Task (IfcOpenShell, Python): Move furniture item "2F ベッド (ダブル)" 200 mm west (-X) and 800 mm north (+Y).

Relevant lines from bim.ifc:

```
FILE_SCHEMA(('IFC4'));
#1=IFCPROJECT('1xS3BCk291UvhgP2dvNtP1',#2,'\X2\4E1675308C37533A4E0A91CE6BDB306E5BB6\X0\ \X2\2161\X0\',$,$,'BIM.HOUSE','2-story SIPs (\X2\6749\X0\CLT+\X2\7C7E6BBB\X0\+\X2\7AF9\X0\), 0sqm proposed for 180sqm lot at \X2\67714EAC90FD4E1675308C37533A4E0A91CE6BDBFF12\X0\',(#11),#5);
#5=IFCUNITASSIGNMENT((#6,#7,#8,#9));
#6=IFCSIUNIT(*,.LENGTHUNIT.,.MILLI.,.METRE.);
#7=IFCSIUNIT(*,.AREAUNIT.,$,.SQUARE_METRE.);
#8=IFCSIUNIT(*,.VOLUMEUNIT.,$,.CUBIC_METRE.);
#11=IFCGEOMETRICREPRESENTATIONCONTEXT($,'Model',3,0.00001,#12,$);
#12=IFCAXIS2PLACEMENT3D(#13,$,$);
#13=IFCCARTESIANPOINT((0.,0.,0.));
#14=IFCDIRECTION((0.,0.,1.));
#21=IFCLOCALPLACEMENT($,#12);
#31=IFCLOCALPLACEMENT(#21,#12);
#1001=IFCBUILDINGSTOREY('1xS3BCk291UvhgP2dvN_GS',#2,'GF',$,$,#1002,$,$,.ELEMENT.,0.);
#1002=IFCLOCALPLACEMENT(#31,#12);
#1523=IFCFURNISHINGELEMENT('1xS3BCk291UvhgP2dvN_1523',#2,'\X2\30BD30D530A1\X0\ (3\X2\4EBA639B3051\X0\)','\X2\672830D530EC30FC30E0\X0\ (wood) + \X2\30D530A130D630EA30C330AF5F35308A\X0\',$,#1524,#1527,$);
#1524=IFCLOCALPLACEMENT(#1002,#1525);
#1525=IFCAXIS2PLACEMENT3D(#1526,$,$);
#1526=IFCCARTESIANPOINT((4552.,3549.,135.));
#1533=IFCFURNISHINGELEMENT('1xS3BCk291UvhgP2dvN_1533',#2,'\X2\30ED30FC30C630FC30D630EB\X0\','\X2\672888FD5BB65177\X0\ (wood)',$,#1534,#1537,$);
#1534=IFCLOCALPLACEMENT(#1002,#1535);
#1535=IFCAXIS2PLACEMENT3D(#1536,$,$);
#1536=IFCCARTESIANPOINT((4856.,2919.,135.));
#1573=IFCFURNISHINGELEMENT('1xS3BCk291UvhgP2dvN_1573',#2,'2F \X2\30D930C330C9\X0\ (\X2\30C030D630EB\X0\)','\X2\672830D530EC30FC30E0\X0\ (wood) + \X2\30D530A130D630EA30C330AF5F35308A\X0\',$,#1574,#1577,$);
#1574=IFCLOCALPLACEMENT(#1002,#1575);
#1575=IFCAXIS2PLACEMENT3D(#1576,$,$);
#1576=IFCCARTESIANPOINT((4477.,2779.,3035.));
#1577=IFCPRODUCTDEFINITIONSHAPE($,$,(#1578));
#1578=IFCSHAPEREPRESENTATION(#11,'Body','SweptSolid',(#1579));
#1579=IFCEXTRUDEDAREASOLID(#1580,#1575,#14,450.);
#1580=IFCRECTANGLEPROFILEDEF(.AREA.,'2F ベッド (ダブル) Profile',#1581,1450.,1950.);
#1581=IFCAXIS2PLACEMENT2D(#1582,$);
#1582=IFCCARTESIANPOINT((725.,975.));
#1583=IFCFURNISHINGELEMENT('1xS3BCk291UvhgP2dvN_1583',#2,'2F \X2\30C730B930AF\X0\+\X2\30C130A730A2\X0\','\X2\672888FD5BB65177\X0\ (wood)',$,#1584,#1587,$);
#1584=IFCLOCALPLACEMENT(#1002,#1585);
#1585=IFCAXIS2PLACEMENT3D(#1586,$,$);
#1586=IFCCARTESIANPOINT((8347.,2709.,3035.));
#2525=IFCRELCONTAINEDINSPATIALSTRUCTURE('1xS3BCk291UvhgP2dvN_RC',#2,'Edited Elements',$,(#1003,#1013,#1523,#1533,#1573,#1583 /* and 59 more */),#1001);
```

```python
import ifcopenshell
import ifcopenshell.api.geometry
import ifcopenshell.util.placement
import ifcopenshell.util.unit

model = ifcopenshell.open("bim.ifc")
unit_scale = ifcopenshell.util.unit.calculate_unit_scale(model)

item = model.by_guid("1xS3BCk291UvhgP2dvN_1573")
matrix = ifcopenshell.util.placement.get_local_placement(item.ObjectPlacement)
matrix[0, 3] -= 0.2 / unit_scale
matrix[1, 3] += 0.8 / unit_scale
ifcopenshell.api.geometry.edit_object_placement(model, product=item, matrix=matrix, is_si=False)

print(ifcopenshell.util.placement.get_local_placement(item.ObjectPlacement).round(3) + 0.0)

model.write("bim_edited.ifc")
```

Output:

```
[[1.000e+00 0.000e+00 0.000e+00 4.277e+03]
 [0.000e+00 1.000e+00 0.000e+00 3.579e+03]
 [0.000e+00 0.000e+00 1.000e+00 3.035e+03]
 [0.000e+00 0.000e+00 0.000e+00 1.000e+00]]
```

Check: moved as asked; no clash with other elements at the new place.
